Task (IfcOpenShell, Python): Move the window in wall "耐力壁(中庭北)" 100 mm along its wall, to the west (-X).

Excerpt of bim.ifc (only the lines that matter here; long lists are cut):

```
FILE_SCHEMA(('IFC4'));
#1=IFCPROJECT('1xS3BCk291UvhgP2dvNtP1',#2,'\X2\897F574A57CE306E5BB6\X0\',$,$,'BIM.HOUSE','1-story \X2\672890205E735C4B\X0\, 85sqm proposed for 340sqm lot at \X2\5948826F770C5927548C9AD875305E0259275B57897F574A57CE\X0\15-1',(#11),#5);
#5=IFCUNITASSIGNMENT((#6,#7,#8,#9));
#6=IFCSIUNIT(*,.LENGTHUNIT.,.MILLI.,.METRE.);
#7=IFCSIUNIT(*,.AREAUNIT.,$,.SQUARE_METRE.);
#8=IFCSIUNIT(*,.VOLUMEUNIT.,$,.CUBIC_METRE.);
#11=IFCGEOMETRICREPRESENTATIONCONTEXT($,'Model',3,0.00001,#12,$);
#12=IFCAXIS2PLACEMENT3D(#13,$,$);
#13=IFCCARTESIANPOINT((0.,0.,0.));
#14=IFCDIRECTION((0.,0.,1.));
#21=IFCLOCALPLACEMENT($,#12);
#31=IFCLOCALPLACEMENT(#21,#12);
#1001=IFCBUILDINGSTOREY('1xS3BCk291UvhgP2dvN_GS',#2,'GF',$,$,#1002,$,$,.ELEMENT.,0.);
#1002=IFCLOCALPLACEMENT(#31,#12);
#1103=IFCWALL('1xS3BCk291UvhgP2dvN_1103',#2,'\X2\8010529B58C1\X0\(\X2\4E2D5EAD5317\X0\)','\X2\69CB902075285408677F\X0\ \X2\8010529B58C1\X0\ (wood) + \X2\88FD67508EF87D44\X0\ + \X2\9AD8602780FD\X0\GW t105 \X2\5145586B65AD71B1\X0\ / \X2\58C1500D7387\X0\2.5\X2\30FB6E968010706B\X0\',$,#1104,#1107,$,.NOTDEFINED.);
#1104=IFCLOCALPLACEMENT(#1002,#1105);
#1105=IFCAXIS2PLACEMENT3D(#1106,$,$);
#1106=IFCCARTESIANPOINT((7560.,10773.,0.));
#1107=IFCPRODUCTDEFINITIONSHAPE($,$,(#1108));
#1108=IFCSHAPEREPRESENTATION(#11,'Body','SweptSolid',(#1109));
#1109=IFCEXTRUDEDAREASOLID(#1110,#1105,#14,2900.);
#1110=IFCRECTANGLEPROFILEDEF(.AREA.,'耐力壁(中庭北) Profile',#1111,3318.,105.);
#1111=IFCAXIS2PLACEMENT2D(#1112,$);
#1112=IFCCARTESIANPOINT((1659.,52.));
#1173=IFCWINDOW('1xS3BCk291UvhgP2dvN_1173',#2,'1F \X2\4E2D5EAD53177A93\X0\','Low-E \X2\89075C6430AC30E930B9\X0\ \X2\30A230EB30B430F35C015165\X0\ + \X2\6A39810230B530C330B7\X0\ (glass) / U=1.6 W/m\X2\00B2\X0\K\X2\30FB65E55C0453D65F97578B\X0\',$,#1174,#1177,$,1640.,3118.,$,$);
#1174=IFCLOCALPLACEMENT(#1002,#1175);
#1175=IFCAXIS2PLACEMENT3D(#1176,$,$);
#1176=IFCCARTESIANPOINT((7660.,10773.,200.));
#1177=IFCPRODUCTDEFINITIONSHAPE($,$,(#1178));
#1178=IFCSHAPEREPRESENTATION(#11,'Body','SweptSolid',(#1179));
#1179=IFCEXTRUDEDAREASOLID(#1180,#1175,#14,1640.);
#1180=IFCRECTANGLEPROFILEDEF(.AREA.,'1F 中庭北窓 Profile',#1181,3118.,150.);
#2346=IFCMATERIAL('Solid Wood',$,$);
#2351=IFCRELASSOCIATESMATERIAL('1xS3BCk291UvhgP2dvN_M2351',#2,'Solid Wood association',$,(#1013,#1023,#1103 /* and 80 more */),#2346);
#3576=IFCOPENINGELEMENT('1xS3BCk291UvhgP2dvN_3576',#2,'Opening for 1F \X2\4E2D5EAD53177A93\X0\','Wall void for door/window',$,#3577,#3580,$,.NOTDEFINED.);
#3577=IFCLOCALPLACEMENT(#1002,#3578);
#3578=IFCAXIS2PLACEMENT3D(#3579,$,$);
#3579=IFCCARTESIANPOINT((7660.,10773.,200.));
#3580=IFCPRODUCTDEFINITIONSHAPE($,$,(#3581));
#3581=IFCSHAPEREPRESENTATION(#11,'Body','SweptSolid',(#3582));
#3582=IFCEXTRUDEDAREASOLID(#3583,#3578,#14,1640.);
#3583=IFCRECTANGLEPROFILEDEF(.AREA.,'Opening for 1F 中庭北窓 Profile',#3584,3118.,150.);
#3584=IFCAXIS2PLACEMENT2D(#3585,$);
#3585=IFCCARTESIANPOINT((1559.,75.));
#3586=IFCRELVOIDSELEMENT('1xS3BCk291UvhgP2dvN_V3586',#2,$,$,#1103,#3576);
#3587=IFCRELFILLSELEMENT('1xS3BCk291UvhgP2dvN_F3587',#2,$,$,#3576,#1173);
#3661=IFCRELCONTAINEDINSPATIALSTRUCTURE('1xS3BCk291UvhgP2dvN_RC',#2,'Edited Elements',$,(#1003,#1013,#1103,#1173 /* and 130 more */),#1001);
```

```python
import ifcopenshell
import ifcopenshell.api.geometry
import ifcopenshell.util.placement
import ifcopenshell.util.unit

model = ifcopenshell.open("bim.ifc")
unit_scale = ifcopenshell.util.unit.calculate_unit_scale(model)

window = model.by_guid("1xS3BCk291UvhgP2dvN_1173")
opening = window.FillsVoids[0].RelatingOpeningElement
wall = opening.VoidsElements[0].RelatingBuildingElement

wall_matrix = ifcopenshell.util.placement.get_local_placement(wall.ObjectPlacement)
shift = wall_matrix[:3, 0] * -0.1 / unit_scale
before = ifcopenshell.util.placement.get_local_placement(window.ObjectPlacement)[:3, 3].copy()

# The window is not placed relative to its opening, so move both.
for product in (opening, window):
    matrix = ifcopenshell.util.placement.get_local_placement(product.ObjectPlacement)
    matrix[:3, 3] += shift
    ifcopenshell.api.geometry.edit_object_placement(model, product=product, matrix=matrix, is_si=False)

after = ifcopenshell.util.placement.get_local_placement(window.ObjectPlacement)[:3, 3]
print("window moved by", (after - before).round(3) + 0.0)

model.write("bim_v2.ifc")
```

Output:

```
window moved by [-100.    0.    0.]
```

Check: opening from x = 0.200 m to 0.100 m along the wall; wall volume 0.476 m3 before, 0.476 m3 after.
